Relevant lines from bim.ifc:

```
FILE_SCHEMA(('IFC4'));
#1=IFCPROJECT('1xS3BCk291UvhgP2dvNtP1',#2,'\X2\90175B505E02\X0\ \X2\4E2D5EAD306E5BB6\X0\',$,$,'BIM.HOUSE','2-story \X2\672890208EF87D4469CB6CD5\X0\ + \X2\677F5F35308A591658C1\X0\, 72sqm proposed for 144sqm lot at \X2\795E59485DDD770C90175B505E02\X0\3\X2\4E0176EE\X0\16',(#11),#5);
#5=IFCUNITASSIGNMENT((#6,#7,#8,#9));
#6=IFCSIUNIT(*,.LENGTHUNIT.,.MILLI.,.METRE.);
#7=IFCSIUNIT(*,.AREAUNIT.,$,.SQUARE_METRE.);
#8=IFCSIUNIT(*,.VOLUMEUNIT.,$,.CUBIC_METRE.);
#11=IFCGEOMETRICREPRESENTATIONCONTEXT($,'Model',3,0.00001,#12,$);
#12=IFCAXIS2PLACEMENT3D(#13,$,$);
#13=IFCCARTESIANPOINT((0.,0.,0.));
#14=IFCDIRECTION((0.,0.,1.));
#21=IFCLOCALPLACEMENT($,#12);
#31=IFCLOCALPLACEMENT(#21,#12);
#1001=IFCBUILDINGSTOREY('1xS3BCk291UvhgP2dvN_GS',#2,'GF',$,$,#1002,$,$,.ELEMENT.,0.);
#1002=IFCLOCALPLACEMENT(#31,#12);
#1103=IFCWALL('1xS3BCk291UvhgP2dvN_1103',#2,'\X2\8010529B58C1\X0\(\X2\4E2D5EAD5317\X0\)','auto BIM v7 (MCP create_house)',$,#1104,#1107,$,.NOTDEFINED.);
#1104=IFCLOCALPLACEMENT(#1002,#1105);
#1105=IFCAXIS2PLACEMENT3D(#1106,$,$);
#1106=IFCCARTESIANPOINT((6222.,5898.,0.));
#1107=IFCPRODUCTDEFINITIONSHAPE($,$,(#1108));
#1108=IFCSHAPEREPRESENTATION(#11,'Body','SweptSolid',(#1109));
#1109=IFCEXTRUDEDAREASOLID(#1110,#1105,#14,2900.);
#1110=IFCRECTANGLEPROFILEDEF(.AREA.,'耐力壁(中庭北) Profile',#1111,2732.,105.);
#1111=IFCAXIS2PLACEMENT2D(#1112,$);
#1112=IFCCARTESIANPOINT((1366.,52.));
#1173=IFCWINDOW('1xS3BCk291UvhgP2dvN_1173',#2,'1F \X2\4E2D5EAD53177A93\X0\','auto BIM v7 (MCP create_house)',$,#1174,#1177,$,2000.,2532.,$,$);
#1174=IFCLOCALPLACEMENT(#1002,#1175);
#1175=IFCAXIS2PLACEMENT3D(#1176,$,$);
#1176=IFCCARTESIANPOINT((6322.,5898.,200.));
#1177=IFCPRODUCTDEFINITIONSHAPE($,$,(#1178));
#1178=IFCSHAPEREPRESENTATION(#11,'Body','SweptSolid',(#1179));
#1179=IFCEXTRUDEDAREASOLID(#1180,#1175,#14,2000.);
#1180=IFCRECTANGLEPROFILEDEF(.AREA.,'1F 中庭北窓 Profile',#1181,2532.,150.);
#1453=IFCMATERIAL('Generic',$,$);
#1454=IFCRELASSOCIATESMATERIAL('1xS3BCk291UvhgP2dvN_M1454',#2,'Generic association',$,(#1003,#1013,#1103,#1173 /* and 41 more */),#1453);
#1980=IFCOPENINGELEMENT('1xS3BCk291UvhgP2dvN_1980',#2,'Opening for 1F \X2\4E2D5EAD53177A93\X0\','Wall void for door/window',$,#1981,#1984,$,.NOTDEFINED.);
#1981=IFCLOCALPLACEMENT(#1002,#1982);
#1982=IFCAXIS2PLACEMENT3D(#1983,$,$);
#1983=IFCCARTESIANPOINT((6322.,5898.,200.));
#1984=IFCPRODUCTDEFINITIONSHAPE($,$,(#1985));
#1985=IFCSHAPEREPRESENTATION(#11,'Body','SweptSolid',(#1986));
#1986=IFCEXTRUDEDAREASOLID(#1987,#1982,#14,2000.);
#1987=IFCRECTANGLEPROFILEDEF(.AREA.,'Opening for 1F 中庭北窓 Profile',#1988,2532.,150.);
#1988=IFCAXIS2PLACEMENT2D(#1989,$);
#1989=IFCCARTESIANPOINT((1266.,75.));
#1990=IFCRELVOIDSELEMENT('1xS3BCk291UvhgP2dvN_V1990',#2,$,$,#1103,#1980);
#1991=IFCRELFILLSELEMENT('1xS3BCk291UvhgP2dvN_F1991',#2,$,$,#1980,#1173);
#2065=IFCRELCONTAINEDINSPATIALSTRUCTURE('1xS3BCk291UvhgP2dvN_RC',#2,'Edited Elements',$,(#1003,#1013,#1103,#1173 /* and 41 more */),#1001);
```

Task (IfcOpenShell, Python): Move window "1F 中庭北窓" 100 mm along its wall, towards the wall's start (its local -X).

```python
import ifcopenshell
import ifcopenshell.api.geometry
import ifcopenshell.util.placement
import ifcopenshell.util.unit

model = ifcopenshell.open("bim.ifc")
unit_scale = ifcopenshell.util.unit.calculate_unit_scale(model)

window = model.by_guid("1xS3BCk291UvhgP2dvN_1173")
opening = window.FillsVoids[0].RelatingOpeningElement
wall = opening.VoidsElements[0].RelatingBuildingElement

wall_matrix = ifcopenshell.util.placement.get_local_placement(wall.ObjectPlacement)
shift = wall_matrix[:3, 0] * -0.1 / unit_scale
before = ifcopenshell.util.placement.get_local_placement(window.ObjectPlacement)[:3, 3].copy()

# The window is not placed relative to its opening, so move both.
for product in (opening, window):
    matrix = ifcopenshell.util.placement.get_local_placement(product.ObjectPlacement)
    matrix[:3, 3] += shift
    ifcopenshell.api.geometry.edit_object_placement(model, product=product, matrix=matrix, is_si=False)

after = ifcopenshell.util.placement.get_local_placement(window.ObjectPlacement)[:3, 3]
print("window moved by", (after - before).round(3) + 0.0)

model.write("bim_rev.ifc")
```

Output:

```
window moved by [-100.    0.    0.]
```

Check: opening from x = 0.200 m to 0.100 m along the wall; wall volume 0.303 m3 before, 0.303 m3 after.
